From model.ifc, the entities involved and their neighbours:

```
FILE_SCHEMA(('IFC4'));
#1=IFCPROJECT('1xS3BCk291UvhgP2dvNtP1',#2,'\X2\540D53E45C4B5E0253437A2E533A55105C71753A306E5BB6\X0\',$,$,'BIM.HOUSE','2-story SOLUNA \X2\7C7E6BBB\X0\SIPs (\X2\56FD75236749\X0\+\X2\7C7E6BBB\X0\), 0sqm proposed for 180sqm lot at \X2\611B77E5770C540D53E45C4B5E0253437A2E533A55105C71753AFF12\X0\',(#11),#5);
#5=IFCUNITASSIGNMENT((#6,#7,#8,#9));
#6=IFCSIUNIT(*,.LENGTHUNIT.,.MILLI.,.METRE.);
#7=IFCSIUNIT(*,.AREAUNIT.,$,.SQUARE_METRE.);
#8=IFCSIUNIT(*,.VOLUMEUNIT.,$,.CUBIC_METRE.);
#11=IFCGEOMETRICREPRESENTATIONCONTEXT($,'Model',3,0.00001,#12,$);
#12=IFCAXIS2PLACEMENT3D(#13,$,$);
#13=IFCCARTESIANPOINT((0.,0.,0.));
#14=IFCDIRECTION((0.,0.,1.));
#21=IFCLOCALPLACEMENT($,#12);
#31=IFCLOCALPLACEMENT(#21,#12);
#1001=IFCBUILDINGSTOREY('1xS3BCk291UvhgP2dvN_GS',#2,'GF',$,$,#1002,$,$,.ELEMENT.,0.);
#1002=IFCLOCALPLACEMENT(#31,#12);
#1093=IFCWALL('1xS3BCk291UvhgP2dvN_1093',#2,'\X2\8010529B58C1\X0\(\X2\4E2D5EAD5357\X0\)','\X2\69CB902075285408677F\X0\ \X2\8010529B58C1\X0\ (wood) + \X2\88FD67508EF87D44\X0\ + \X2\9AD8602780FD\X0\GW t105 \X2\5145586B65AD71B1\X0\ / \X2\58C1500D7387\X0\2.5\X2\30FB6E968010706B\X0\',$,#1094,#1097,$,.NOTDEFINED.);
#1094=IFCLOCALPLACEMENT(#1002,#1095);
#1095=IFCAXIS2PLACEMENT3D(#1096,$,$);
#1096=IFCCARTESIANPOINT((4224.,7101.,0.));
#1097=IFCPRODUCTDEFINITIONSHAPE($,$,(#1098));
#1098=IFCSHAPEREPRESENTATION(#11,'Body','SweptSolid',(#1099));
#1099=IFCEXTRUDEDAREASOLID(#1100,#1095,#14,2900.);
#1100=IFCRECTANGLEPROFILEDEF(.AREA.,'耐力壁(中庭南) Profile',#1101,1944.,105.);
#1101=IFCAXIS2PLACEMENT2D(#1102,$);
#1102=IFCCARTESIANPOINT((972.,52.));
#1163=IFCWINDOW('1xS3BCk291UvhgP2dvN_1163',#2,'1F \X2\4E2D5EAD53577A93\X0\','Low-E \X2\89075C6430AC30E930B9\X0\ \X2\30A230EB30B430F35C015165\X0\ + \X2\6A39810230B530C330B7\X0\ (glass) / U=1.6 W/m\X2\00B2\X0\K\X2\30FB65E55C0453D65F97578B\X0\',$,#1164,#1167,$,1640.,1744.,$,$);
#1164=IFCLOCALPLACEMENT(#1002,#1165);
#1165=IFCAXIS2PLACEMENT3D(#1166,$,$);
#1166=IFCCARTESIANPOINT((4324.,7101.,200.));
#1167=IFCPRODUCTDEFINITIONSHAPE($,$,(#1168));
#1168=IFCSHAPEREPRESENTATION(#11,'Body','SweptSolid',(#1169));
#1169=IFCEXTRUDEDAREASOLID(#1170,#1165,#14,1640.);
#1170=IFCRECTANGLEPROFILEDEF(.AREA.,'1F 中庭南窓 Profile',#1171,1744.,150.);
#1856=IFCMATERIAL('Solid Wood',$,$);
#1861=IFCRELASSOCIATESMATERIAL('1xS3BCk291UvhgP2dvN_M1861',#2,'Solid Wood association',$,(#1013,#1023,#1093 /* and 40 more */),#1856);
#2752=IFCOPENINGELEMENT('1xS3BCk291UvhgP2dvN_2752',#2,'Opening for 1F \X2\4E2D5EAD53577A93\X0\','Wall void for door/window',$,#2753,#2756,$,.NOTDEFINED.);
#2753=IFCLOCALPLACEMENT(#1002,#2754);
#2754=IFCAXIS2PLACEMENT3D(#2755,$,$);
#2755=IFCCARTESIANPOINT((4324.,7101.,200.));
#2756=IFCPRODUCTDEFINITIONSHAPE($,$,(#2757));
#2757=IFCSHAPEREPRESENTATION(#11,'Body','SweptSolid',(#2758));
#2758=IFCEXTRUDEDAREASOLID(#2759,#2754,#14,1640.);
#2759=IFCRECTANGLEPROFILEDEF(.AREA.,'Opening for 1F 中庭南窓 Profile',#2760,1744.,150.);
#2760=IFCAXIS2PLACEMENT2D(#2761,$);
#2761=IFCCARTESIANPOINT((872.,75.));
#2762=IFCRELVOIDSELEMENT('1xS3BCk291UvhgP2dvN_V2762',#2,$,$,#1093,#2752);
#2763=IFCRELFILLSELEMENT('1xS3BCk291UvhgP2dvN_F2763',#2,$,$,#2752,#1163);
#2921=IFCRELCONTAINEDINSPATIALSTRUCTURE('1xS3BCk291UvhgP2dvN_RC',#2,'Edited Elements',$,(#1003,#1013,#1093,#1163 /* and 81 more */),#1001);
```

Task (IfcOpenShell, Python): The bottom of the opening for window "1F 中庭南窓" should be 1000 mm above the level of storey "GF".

```python
import numpy as np
import ifcopenshell
import ifcopenshell.api.geometry
import ifcopenshell.geom
import ifcopenshell.util.element
import ifcopenshell.util.placement
import ifcopenshell.util.shape
import ifcopenshell.util.unit

model = ifcopenshell.open("model.ifc")
unit_scale = ifcopenshell.util.unit.calculate_unit_scale(model)

window = model.by_id(1163)
opening = window.FillsVoids[0].RelatingOpeningElement
storey = ifcopenshell.util.element.get_container(window, ifc_class="IfcBuildingStorey")
level = ifcopenshell.util.placement.get_local_placement(storey.ObjectPlacement)[2, 3]

# The opening's origin need not be at the sill, so measure its lowest point.
shape = ifcopenshell.geom.create_shape(ifcopenshell.geom.settings(), opening)
bottom = ifcopenshell.util.shape.get_shape_bottom_elevation(shape, shape.geometry) / unit_scale
dz = level + 1000.0 - bottom

shift = np.array([0.0, 0.0, dz])
# The window is not placed relative to its opening, so move both.
for product in (opening, window):
    matrix = ifcopenshell.util.placement.get_local_placement(product.ObjectPlacement)
    matrix[:3, 3] += shift
    ifcopenshell.api.geometry.edit_object_placement(model, product=product, matrix=matrix, is_si=False)

print(f"moved by {dz * unit_scale:+.3f} m")

model.write("model-out.ifc")
```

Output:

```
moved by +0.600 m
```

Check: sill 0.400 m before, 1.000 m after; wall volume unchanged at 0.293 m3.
